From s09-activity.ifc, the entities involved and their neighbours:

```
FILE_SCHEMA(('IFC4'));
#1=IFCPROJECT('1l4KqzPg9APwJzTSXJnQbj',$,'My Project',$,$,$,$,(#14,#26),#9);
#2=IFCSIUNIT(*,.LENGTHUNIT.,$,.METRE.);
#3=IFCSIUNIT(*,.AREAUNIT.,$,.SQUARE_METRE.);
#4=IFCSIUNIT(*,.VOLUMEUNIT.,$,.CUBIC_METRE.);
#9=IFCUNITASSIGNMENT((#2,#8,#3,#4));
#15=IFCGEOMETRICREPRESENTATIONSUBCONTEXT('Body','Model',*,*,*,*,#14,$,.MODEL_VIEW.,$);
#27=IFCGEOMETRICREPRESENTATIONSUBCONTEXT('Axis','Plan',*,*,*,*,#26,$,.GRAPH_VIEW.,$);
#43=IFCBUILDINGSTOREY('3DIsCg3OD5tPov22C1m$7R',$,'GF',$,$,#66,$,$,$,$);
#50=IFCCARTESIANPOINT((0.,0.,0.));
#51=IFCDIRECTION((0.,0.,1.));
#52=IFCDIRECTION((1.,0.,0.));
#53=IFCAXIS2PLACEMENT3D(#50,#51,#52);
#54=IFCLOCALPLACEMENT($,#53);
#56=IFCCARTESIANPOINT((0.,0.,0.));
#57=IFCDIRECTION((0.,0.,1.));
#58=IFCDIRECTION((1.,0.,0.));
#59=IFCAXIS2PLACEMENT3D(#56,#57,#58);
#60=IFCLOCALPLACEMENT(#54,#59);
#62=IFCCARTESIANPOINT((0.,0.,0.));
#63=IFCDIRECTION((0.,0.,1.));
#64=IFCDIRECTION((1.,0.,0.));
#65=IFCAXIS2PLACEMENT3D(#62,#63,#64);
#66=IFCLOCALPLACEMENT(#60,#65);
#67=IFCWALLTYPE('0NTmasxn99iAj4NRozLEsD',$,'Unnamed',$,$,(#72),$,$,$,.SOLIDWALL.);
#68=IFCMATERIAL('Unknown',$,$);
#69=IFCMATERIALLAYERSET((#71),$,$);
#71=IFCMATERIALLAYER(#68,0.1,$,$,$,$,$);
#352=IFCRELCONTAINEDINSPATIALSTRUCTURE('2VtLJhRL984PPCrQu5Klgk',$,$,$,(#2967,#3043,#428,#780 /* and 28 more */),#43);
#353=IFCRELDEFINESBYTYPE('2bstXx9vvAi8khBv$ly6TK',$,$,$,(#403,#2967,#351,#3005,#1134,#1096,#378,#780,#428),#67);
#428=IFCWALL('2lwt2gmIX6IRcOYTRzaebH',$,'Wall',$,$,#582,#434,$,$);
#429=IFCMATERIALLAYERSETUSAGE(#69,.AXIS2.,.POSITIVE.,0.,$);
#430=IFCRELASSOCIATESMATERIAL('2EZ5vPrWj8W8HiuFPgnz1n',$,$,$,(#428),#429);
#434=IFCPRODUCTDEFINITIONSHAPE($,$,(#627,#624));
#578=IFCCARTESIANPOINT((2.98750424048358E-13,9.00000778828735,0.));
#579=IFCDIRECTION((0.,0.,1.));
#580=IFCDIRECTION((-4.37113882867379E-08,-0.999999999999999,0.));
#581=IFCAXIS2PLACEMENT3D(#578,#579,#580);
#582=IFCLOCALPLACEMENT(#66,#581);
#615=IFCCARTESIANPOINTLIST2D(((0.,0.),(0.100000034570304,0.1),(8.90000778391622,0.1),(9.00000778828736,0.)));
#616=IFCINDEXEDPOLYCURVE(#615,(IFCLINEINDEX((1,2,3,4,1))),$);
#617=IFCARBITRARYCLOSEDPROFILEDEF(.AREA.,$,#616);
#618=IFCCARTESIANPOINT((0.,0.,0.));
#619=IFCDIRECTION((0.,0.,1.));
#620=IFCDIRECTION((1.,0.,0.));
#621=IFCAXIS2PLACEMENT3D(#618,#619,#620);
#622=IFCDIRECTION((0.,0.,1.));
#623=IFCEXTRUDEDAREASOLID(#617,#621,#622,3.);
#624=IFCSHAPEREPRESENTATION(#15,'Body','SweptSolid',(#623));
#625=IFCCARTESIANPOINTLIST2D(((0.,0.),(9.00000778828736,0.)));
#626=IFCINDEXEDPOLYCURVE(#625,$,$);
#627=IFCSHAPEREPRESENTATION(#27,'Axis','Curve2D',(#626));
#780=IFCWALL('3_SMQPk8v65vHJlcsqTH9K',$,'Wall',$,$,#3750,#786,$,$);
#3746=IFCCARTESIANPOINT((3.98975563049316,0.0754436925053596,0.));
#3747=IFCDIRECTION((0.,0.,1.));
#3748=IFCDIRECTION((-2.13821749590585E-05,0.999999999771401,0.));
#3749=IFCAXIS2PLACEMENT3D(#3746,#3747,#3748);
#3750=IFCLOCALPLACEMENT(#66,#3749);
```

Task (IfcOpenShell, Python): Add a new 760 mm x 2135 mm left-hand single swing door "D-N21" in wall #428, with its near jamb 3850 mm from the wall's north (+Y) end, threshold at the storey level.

```python
import numpy as np
import ifcopenshell
import ifcopenshell.api.feature
import ifcopenshell.api.geometry
import ifcopenshell.api.root
import ifcopenshell.api.spatial
import ifcopenshell.geom
import ifcopenshell.util.element
import ifcopenshell.util.placement
import ifcopenshell.util.representation
import ifcopenshell.util.shape
import ifcopenshell.util.unit

model = ifcopenshell.open("s09-activity.ifc")
unit_scale = ifcopenshell.util.unit.calculate_unit_scale(model)
settings = ifcopenshell.geom.settings()


def volume(element):
    """Net volume in cubic metres, openings subtracted."""
    shape = ifcopenshell.geom.create_shape(settings, element)
    return ifcopenshell.util.shape.get_volume(shape.geometry)


wall = model.by_id(428)
storey = ifcopenshell.util.element.get_container(wall, ifc_class="IfcBuildingStorey")
context = ifcopenshell.util.representation.get_context(model, "Model", "Body", "MODEL_VIEW")
before = volume(wall)

width, height, from_end, sill = 0.76, 2.135, 3.85, 0.0  # metres

# The wall runs along its own X axis, and the end named is its -X end.
wall_shape = ifcopenshell.geom.create_shape(settings, wall)
x, y, z = ifcopenshell.util.shape.get_vertices(wall_shape.geometry).T
start = x.min() + from_end
face, thickness = float(y.min()), float(y.max() - y.min())
wall_matrix = ifcopenshell.util.placement.get_local_placement(wall.ObjectPlacement)
level = ifcopenshell.util.placement.get_local_placement(storey.ObjectPlacement)[2, 3]


def in_wall(x, y):
    """Placement at x, y metres in the wall's axes, at sill height."""
    matrix = wall_matrix.copy()
    matrix[:, 3] = wall_matrix @ np.array([x / unit_scale, y / unit_scale, 0.0, 1.0])
    matrix[2, 3] = level + sill / unit_scale
    return matrix


# Opening: a box that overshoots both wall faces by 50 mm.
opening = ifcopenshell.api.root.create_entity(model, ifc_class="IfcOpeningElement", predefined_type="OPENING")
box = ifcopenshell.api.geometry.add_wall_representation(
    model, context=context, length=width, height=height, thickness=thickness + 0.1
)
ifcopenshell.api.geometry.assign_representation(model, product=opening, representation=box)
ifcopenshell.api.geometry.edit_object_placement(model, product=opening, matrix=in_wall(start, face - 0.05), is_si=False)
ifcopenshell.api.feature.add_feature(model, feature=opening, element=wall)

door = ifcopenshell.api.root.create_entity(model, ifc_class="IfcDoor", name="D-N21", predefined_type="DOOR")
door.OverallWidth, door.OverallHeight = width / unit_scale, height / unit_scale
door.OperationType = "SINGLE_SWING_LEFT"
body = ifcopenshell.api.geometry.add_door_representation(
    model,
    context=context,
    overall_width=door.OverallWidth,
    overall_height=door.OverallHeight,
    operation_type="SINGLE_SWING_LEFT",
    lining_properties={"LiningDepth": thickness / unit_scale, "ThresholdDepth": thickness / unit_scale},
)
ifcopenshell.api.geometry.assign_representation(model, product=door, representation=body)
ifcopenshell.api.spatial.assign_container(model, products=[door], relating_structure=storey)
ifcopenshell.api.feature.add_filling(model, opening=opening, element=door)

# The lining spans the wall, so the door starts at the wall face.
ifcopenshell.api.geometry.edit_object_placement(model, product=door, matrix=in_wall(start, face), is_si=False)

after = volume(wall)

print(f"wall volume {before:.3f} -> {after:.3f} m3")

model.write("s09-activity-out.ifc")
```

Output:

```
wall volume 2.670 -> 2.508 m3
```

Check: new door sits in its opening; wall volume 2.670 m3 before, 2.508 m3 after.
